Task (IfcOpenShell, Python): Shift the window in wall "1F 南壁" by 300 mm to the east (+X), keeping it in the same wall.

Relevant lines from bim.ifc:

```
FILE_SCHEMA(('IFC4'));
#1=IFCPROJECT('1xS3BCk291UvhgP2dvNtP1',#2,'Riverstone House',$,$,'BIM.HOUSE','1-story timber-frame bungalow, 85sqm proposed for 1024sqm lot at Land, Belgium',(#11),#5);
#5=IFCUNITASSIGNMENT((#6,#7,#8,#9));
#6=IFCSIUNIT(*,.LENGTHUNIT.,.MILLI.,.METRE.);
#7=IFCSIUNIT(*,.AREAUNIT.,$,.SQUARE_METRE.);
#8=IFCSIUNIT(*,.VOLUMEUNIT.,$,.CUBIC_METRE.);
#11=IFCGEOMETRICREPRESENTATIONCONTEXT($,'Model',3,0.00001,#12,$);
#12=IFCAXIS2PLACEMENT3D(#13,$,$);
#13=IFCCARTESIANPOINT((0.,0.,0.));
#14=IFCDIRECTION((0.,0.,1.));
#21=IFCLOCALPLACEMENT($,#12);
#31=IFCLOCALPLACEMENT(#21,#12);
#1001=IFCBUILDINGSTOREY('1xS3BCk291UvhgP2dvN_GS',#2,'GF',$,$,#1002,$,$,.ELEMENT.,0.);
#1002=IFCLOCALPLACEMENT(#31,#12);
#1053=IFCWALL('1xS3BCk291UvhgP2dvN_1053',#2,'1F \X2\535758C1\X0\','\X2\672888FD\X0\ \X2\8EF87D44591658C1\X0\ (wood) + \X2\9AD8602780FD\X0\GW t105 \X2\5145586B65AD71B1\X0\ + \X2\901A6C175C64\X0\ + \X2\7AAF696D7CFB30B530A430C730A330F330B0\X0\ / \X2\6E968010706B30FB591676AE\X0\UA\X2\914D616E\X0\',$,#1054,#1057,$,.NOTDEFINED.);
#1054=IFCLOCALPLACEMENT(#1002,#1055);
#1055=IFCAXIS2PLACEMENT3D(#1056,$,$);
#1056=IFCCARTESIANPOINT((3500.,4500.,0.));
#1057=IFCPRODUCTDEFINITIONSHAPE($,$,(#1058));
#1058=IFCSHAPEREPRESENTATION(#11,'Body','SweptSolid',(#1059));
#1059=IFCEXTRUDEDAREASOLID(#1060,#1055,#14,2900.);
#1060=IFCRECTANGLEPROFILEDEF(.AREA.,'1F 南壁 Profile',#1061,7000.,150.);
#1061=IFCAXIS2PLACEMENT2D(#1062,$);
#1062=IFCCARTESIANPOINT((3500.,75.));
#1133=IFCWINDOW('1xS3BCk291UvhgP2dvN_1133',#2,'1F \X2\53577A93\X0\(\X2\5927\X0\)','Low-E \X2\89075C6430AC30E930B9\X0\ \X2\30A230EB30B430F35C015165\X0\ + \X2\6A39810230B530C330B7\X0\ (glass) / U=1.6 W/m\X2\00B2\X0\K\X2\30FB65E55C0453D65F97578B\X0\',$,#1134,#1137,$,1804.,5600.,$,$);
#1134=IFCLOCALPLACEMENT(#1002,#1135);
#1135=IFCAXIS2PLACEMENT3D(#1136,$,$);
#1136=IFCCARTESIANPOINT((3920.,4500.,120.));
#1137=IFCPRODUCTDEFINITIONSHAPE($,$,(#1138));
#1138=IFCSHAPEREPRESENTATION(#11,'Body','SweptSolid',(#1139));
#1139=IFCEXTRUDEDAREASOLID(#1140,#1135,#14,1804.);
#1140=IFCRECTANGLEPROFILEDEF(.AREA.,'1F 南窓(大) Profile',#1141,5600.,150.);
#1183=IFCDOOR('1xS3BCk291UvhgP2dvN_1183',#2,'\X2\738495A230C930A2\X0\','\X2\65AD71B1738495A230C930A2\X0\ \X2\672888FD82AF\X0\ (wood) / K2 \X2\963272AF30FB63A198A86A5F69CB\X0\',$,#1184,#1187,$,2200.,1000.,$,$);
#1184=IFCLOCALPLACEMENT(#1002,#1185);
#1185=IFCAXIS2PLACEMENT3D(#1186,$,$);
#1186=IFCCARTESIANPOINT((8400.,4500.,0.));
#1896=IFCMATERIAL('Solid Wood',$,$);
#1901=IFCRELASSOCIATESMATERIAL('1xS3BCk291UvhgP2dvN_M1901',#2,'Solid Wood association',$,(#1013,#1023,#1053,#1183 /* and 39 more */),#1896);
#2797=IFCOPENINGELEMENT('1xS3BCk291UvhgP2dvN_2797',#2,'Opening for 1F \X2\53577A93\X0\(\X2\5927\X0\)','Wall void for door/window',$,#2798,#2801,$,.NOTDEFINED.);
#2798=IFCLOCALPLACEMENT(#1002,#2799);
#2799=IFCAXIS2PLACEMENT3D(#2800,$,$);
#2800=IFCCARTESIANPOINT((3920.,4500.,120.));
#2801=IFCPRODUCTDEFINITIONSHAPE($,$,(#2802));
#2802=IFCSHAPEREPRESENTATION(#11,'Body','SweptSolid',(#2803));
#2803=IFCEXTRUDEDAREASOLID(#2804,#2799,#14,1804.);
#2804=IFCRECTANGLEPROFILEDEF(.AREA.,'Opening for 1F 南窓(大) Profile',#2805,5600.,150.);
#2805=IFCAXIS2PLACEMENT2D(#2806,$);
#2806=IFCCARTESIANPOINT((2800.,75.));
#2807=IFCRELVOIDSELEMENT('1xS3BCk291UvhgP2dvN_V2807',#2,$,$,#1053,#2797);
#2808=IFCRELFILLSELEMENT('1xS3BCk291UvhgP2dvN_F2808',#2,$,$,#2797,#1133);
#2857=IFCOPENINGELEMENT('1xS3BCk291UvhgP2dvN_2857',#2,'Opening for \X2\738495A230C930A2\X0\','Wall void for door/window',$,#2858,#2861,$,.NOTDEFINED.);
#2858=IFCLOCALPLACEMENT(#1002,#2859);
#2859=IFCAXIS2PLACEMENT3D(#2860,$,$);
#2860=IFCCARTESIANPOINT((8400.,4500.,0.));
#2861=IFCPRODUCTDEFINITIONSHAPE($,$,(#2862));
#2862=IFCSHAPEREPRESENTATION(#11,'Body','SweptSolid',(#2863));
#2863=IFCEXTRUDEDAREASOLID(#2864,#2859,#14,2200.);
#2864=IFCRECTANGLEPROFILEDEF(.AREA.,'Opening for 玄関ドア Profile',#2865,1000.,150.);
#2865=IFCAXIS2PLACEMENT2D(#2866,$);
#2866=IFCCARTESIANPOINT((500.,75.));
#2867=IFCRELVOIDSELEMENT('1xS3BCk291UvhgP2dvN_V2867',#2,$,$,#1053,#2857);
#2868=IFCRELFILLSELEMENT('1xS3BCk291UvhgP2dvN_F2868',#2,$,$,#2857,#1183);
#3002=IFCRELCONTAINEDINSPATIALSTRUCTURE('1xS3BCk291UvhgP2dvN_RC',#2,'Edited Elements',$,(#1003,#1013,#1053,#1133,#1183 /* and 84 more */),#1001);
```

```python
import ifcopenshell
import ifcopenshell.api.geometry
import ifcopenshell.util.placement
import ifcopenshell.util.unit

model = ifcopenshell.open("bim.ifc")
unit_scale = ifcopenshell.util.unit.calculate_unit_scale(model)

window = model.by_guid("1xS3BCk291UvhgP2dvN_1133")
opening = window.FillsVoids[0].RelatingOpeningElement
wall = opening.VoidsElements[0].RelatingBuildingElement

wall_matrix = ifcopenshell.util.placement.get_local_placement(wall.ObjectPlacement)
shift = wall_matrix[:3, 0] * 0.3 / unit_scale
before = ifcopenshell.util.placement.get_local_placement(window.ObjectPlacement)[:3, 3].copy()

# The window is not placed relative to its opening, so move both.
for product in (opening, window):
    matrix = ifcopenshell.util.placement.get_local_placement(product.ObjectPlacement)
    matrix[:3, 3] += shift
    ifcopenshell.api.geometry.edit_object_placement(model, product=product, matrix=matrix, is_si=False)

after = ifcopenshell.util.placement.get_local_placement(window.ObjectPlacement)[:3, 3]
print("window moved by", (after - before).round(3) + 0.0)

model.write("bim_rev.ifc")
```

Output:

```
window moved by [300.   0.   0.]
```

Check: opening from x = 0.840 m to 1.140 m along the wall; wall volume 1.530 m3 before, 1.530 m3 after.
